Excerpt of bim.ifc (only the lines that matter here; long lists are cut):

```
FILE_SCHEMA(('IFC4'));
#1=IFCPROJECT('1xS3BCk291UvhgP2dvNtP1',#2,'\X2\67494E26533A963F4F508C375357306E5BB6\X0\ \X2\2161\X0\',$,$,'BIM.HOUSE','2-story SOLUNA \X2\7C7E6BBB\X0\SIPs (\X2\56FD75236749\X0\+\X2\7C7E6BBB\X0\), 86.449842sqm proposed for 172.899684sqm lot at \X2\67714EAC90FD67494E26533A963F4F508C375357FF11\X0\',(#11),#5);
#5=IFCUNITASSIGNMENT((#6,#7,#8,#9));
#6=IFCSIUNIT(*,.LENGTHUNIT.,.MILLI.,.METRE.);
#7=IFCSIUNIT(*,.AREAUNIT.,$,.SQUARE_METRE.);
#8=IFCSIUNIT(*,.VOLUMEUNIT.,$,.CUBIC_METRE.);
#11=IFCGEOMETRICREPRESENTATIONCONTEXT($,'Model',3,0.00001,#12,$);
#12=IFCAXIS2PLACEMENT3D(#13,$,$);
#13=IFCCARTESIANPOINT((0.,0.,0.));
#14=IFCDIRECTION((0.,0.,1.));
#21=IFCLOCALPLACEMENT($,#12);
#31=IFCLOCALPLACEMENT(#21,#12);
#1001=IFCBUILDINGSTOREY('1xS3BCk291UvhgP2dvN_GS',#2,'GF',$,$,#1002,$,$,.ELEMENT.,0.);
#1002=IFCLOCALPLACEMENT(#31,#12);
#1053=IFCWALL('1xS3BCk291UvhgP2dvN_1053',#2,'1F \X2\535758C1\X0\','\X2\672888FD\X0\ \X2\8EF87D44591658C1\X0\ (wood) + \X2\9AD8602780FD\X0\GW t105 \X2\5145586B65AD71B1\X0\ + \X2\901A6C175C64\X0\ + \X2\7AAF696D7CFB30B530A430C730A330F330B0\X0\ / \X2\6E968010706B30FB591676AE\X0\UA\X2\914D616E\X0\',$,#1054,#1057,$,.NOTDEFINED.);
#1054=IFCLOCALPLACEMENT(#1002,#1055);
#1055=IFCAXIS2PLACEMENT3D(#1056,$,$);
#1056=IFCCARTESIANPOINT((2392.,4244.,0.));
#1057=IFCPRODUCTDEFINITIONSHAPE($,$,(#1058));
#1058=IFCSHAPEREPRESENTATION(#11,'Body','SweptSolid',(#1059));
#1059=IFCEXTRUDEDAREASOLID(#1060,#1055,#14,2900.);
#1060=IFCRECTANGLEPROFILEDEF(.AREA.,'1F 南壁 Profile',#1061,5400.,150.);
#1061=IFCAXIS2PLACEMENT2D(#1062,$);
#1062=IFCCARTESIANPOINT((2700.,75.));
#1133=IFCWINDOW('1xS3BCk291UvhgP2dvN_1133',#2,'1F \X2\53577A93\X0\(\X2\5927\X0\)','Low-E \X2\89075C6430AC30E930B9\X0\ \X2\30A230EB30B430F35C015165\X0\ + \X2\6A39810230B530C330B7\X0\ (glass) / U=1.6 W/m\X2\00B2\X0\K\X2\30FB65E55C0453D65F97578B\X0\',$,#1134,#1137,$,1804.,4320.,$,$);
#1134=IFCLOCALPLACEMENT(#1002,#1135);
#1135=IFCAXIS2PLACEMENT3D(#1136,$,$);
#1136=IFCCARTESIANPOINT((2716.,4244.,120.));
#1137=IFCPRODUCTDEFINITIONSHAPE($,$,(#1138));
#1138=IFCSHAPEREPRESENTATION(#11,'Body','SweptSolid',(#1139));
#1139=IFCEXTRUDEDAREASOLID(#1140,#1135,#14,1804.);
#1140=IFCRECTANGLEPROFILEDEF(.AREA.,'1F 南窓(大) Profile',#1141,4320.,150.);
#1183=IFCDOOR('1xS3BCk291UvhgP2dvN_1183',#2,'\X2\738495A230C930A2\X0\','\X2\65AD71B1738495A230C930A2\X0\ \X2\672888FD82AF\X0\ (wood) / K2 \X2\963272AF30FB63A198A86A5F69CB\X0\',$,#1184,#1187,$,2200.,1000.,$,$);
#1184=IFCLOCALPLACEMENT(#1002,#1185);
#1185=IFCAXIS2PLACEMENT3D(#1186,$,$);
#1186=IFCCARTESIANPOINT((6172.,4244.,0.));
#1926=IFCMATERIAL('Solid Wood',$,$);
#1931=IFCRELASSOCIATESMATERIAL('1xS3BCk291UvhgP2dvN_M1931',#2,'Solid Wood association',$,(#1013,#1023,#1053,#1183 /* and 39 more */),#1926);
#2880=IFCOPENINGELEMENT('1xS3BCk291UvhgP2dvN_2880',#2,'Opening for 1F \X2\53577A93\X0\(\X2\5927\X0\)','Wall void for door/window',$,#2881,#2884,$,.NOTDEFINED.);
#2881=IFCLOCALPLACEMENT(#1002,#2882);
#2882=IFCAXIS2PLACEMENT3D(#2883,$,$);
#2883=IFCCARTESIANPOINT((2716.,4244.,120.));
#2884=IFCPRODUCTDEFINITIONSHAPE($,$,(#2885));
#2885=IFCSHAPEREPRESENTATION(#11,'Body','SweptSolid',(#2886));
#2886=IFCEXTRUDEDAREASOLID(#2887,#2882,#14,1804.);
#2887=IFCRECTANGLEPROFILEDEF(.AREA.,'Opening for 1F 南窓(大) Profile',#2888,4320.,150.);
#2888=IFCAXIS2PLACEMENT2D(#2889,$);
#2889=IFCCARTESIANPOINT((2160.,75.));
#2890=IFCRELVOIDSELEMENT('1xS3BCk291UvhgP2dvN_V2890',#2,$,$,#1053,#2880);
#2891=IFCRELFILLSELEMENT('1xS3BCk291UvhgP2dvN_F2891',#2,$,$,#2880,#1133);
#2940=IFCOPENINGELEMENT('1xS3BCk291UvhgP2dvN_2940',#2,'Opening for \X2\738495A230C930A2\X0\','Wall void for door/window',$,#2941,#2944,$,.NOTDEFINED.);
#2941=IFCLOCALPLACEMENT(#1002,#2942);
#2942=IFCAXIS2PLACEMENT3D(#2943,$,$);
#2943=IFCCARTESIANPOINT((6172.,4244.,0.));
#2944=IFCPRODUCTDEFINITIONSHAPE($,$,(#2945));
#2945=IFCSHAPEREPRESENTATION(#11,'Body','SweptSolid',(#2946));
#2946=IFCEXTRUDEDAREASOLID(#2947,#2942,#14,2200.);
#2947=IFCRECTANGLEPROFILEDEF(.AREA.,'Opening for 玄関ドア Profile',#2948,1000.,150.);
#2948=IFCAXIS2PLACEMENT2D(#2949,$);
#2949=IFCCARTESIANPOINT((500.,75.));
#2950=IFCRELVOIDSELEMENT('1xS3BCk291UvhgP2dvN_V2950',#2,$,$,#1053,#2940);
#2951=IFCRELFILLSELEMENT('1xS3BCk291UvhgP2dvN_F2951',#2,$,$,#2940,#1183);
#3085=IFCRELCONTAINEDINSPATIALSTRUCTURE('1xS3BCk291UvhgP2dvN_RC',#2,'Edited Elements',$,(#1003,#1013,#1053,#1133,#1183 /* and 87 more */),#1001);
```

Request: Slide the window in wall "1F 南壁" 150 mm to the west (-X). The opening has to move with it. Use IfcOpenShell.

```python
import ifcopenshell
import ifcopenshell.api.geometry
import ifcopenshell.util.placement
import ifcopenshell.util.unit

model = ifcopenshell.open("bim.ifc")
unit_scale = ifcopenshell.util.unit.calculate_unit_scale(model)

window = model.by_guid("1xS3BCk291UvhgP2dvN_1133")
opening = window.FillsVoids[0].RelatingOpeningElement
wall = opening.VoidsElements[0].RelatingBuildingElement

wall_matrix = ifcopenshell.util.placement.get_local_placement(wall.ObjectPlacement)
shift = wall_matrix[:3, 0] * -0.15 / unit_scale
before = ifcopenshell.util.placement.get_local_placement(window.ObjectPlacement)[:3, 3].copy()

# The window is not placed relative to its opening, so move both.
for product in (opening, window):
    matrix = ifcopenshell.util.placement.get_local_placement(product.ObjectPlacement)
    matrix[:3, 3] += shift
    ifcopenshell.api.geometry.edit_object_placement(model, product=product, matrix=matrix, is_si=False)

after = ifcopenshell.util.placement.get_local_placement(window.ObjectPlacement)[:3, 3]
print("window moved by", (after - before).round(3) + 0.0)

model.write("bim_edited.ifc")
```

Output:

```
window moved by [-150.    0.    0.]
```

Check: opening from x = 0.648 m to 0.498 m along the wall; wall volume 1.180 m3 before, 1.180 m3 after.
